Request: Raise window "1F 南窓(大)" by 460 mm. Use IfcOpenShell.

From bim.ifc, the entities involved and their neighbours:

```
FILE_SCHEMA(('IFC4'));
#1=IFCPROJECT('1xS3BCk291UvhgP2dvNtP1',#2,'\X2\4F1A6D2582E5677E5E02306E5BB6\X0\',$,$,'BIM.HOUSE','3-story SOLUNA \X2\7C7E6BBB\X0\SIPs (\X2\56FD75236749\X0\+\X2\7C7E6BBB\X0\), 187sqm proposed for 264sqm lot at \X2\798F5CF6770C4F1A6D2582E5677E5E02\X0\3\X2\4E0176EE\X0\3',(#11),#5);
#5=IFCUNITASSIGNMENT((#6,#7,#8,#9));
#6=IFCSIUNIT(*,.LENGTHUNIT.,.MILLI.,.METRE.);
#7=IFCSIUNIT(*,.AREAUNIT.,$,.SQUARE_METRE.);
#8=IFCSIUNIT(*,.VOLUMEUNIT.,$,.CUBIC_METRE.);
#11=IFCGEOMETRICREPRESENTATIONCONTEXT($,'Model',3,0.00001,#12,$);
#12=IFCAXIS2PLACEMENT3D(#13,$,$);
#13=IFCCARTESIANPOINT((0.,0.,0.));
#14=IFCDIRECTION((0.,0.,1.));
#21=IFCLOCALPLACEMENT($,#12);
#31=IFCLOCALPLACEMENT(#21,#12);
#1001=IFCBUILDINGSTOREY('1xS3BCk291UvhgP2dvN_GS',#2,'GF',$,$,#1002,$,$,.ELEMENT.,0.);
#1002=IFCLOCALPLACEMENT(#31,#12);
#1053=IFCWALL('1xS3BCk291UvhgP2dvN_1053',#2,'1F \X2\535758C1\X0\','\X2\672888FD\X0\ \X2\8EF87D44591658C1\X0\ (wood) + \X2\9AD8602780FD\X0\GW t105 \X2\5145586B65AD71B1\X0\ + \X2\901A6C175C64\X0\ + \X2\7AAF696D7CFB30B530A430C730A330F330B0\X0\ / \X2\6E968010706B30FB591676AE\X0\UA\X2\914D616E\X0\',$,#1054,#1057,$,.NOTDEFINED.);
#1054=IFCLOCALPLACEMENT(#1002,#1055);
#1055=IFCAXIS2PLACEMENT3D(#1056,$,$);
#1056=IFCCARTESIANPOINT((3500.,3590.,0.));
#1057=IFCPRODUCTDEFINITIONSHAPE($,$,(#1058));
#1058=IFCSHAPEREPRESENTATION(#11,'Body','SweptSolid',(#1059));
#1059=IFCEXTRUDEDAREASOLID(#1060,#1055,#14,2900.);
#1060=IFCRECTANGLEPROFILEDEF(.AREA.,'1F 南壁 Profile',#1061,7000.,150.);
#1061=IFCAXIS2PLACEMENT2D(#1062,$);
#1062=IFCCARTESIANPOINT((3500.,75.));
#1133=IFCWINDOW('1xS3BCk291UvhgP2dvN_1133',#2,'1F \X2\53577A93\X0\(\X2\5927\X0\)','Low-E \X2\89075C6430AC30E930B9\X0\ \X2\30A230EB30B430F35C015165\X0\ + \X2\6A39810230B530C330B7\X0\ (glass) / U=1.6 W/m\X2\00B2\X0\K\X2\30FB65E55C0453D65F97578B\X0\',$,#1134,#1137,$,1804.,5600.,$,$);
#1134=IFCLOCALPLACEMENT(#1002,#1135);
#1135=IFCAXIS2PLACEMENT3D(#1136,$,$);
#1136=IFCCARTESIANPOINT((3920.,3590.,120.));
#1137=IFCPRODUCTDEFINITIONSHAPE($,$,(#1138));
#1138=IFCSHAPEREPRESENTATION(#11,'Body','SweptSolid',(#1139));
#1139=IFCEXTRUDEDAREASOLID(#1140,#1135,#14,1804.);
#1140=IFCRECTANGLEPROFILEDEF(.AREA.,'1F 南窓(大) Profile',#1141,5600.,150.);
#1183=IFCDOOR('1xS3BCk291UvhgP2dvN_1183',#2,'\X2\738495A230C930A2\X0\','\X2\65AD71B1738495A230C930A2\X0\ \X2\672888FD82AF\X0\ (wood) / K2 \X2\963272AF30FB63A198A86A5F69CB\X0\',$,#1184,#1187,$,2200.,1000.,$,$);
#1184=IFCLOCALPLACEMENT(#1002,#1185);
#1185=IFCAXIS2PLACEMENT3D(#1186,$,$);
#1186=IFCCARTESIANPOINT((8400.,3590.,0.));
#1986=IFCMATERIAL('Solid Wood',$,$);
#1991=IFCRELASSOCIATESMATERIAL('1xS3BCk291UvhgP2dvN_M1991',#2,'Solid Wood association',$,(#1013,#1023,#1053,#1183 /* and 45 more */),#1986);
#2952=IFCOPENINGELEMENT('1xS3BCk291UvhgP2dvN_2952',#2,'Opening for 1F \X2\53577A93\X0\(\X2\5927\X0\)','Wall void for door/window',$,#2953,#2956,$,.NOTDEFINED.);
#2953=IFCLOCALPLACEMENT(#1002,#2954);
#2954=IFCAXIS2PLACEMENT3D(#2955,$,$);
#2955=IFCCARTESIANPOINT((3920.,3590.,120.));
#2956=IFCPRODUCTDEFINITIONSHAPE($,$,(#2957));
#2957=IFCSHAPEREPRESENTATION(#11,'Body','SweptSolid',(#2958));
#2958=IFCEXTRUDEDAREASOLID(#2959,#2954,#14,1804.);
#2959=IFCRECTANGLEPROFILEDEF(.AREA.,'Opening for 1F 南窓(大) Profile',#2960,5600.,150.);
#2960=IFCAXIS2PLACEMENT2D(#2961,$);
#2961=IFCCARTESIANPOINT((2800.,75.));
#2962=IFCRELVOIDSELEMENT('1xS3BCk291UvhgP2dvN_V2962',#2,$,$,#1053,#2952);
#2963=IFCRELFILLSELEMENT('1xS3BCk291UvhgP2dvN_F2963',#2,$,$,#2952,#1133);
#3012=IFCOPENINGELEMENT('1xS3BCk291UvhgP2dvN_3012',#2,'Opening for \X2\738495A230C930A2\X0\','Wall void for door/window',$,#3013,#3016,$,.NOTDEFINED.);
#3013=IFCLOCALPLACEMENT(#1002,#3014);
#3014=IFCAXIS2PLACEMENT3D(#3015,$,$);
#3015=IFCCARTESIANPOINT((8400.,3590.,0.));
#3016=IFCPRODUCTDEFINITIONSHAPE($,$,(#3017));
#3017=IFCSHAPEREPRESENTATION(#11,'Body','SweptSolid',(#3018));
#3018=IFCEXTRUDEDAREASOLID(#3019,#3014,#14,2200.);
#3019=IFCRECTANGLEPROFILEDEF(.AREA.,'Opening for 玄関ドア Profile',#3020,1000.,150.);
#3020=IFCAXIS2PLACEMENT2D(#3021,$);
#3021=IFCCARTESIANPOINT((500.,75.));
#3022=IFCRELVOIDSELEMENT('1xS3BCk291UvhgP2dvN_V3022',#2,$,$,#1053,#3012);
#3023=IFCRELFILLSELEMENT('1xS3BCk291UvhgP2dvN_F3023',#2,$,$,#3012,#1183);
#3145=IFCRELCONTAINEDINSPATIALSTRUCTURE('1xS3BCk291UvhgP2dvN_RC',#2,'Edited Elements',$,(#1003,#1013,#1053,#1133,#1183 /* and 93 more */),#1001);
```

```python
import numpy as np
import ifcopenshell
import ifcopenshell.api.geometry
import ifcopenshell.util.placement
import ifcopenshell.util.unit

model = ifcopenshell.open("bim.ifc")
unit_scale = ifcopenshell.util.unit.calculate_unit_scale(model)

window = model.by_guid("1xS3BCk291UvhgP2dvN_1133")
opening = window.FillsVoids[0].RelatingOpeningElement
dz = 0.46 / unit_scale

shift = np.array([0.0, 0.0, dz])
# The window is not placed relative to its opening, so move both.
for product in (opening, window):
    matrix = ifcopenshell.util.placement.get_local_placement(product.ObjectPlacement)
    matrix[:3, 3] += shift
    ifcopenshell.api.geometry.edit_object_placement(model, product=product, matrix=matrix, is_si=False)

print(f"moved by {dz * unit_scale:+.3f} m")

model.write("bim-out.ifc")
```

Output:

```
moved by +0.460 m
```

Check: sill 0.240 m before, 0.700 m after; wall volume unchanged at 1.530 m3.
